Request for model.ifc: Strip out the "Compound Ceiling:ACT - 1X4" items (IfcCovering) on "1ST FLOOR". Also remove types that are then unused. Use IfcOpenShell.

First a look at what the model holds.

```python
import ifcopenshell
import ifcopenshell.util.element

model = ifcopenshell.open("model.ifc")
print(model.schema)
storey = next(s for s in model.by_type("IfcBuildingStorey") if s.Name == "1ST FLOOR")
coverings = [e for e in ifcopenshell.util.element.get_decomposition(storey) if e.is_a("IfcCovering")]
seen = {}
for e in coverings:
    element_type = ifcopenshell.util.element.get_type(e)
    name = element_type.Name if element_type not in (None, e) else None
    seen[name] = seen.get(name, 0) + 1
for name, count in sorted(seen.items(), key=str):
    print(count, "x", name)
```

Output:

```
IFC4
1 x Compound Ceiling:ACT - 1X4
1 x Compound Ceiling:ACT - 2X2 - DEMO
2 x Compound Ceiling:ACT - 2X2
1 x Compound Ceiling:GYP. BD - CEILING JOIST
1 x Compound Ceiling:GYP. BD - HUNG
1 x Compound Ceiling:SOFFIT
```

```python
import ifcopenshell
import ifcopenshell.api.root
import ifcopenshell.util.element

model = ifcopenshell.open("model.ifc")

storey = next(s for s in model.by_type("IfcBuildingStorey") if s.Name == "1ST FLOOR")
coverings = [e for e in ifcopenshell.util.element.get_decomposition(storey) if e.is_a("IfcCovering")]
targets = [e for e in coverings if (t := ifcopenshell.util.element.get_type(e)) not in (None, e) and t.Name == "Compound Ceiling:ACT - 1X4"]
types = {ifcopenshell.util.element.get_type(e) for e in targets} - {None, *targets}

for e in targets:
    ifcopenshell.api.root.remove_product(model, product=e)
print(len(targets), "removed")

unused = [t for t in types if not ifcopenshell.util.element.get_types(t)]
for t in unused:
    ifcopenshell.api.root.remove_product(model, product=t)
print(len(unused), "unused types removed")

model.write("model_v2.ifc")
```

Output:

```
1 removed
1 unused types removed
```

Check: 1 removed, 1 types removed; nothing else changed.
